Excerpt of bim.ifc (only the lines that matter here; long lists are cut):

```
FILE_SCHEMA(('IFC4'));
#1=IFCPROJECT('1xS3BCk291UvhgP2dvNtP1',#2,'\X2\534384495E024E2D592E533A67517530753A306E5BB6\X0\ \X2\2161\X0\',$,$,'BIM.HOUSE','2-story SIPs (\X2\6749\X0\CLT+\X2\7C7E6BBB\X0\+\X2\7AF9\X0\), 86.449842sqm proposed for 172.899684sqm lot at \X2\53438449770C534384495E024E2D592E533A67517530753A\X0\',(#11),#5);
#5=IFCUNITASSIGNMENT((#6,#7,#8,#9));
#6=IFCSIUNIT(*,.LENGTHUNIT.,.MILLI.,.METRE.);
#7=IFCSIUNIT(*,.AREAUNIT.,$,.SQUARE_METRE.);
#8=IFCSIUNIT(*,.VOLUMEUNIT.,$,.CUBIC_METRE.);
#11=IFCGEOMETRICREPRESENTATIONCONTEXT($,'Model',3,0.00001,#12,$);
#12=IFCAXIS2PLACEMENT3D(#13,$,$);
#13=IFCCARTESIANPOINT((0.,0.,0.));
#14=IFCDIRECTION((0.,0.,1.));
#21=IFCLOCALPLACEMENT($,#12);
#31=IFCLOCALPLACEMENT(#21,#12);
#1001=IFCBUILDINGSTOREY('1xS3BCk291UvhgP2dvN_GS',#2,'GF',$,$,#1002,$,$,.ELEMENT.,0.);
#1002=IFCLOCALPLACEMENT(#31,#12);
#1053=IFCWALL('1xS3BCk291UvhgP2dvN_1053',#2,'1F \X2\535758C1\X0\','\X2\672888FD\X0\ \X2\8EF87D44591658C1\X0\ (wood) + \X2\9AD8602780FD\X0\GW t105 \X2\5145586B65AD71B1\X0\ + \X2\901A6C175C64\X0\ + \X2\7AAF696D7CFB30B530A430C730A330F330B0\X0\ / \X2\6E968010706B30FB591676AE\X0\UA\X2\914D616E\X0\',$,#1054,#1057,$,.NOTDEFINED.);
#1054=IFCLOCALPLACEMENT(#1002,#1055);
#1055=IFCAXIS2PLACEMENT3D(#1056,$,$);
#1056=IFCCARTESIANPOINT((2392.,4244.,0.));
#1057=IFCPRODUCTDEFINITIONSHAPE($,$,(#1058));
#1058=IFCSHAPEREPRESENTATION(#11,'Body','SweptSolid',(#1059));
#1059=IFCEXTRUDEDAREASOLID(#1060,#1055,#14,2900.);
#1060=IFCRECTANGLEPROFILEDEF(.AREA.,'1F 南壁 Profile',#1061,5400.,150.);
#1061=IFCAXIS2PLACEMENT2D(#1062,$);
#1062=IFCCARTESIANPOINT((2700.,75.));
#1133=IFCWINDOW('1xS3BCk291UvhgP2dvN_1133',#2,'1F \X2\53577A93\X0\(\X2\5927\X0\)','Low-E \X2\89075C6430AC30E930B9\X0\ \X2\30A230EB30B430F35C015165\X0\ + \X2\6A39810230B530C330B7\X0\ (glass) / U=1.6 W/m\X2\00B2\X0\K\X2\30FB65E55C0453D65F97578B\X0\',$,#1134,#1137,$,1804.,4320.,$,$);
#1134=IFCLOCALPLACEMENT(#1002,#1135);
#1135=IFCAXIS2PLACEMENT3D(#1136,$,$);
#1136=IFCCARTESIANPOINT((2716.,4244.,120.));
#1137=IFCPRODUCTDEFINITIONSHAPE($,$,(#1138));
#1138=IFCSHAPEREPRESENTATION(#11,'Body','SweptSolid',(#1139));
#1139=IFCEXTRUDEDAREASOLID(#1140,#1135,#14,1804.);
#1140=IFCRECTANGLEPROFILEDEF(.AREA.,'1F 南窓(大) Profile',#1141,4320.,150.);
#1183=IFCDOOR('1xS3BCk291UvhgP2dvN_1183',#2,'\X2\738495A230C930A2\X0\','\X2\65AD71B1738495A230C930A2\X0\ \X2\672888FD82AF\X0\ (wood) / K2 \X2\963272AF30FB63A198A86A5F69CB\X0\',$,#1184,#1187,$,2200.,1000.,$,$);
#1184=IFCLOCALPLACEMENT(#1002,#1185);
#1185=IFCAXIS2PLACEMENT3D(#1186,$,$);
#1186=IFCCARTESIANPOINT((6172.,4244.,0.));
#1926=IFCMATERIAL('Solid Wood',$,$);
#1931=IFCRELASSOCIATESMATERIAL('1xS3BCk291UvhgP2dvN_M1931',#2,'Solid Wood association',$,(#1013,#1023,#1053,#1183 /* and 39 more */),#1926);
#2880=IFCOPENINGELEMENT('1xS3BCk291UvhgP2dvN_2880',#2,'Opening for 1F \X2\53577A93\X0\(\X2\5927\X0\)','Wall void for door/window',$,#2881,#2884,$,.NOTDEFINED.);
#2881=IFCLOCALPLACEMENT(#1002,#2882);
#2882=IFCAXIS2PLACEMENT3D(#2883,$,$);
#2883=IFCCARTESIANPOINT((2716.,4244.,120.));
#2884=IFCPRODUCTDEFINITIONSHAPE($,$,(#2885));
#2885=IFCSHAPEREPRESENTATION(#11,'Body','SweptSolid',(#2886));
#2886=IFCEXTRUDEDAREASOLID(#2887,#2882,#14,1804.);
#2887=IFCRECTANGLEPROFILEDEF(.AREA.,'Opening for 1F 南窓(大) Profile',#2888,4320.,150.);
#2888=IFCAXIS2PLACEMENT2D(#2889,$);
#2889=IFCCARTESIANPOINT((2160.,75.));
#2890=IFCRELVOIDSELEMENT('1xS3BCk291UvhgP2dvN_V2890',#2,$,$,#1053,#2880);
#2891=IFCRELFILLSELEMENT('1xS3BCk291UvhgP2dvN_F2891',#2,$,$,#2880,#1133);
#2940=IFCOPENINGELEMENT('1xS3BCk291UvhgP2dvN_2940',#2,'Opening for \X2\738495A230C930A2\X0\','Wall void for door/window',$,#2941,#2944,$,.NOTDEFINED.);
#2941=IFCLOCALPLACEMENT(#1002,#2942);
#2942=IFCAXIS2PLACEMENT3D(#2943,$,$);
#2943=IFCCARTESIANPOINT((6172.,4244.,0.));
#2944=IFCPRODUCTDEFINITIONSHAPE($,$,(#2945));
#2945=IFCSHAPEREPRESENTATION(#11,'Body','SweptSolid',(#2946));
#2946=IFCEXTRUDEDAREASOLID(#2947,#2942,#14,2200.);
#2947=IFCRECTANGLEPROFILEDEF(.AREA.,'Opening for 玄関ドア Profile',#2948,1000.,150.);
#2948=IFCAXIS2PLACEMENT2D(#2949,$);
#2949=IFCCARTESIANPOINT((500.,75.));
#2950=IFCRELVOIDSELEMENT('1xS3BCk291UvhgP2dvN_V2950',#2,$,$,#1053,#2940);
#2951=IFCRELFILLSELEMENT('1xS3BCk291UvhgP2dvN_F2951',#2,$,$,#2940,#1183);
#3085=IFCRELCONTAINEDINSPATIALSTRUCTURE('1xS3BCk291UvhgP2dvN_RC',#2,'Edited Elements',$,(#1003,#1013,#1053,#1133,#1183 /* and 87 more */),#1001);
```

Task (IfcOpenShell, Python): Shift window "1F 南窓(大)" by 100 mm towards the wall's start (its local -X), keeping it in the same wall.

```python
import ifcopenshell
import ifcopenshell.api.geometry
import ifcopenshell.util.placement
import ifcopenshell.util.unit

model = ifcopenshell.open("bim.ifc")
unit_scale = ifcopenshell.util.unit.calculate_unit_scale(model)

window = model.by_guid("1xS3BCk291UvhgP2dvN_1133")
opening = window.FillsVoids[0].RelatingOpeningElement
wall = opening.VoidsElements[0].RelatingBuildingElement

wall_matrix = ifcopenshell.util.placement.get_local_placement(wall.ObjectPlacement)
shift = wall_matrix[:3, 0] * -0.1 / unit_scale
before = ifcopenshell.util.placement.get_local_placement(window.ObjectPlacement)[:3, 3].copy()

# The window is not placed relative to its opening, so move both.
for product in (opening, window):
    matrix = ifcopenshell.util.placement.get_local_placement(product.ObjectPlacement)
    matrix[:3, 3] += shift
    ifcopenshell.api.geometry.edit_object_placement(model, product=product, matrix=matrix, is_si=False)

after = ifcopenshell.util.placement.get_local_placement(window.ObjectPlacement)[:3, 3]
print("window moved by", (after - before).round(3) + 0.0)

model.write("bim_edited.ifc")
```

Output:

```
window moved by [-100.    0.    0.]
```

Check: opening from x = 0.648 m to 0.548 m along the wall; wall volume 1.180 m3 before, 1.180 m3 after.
